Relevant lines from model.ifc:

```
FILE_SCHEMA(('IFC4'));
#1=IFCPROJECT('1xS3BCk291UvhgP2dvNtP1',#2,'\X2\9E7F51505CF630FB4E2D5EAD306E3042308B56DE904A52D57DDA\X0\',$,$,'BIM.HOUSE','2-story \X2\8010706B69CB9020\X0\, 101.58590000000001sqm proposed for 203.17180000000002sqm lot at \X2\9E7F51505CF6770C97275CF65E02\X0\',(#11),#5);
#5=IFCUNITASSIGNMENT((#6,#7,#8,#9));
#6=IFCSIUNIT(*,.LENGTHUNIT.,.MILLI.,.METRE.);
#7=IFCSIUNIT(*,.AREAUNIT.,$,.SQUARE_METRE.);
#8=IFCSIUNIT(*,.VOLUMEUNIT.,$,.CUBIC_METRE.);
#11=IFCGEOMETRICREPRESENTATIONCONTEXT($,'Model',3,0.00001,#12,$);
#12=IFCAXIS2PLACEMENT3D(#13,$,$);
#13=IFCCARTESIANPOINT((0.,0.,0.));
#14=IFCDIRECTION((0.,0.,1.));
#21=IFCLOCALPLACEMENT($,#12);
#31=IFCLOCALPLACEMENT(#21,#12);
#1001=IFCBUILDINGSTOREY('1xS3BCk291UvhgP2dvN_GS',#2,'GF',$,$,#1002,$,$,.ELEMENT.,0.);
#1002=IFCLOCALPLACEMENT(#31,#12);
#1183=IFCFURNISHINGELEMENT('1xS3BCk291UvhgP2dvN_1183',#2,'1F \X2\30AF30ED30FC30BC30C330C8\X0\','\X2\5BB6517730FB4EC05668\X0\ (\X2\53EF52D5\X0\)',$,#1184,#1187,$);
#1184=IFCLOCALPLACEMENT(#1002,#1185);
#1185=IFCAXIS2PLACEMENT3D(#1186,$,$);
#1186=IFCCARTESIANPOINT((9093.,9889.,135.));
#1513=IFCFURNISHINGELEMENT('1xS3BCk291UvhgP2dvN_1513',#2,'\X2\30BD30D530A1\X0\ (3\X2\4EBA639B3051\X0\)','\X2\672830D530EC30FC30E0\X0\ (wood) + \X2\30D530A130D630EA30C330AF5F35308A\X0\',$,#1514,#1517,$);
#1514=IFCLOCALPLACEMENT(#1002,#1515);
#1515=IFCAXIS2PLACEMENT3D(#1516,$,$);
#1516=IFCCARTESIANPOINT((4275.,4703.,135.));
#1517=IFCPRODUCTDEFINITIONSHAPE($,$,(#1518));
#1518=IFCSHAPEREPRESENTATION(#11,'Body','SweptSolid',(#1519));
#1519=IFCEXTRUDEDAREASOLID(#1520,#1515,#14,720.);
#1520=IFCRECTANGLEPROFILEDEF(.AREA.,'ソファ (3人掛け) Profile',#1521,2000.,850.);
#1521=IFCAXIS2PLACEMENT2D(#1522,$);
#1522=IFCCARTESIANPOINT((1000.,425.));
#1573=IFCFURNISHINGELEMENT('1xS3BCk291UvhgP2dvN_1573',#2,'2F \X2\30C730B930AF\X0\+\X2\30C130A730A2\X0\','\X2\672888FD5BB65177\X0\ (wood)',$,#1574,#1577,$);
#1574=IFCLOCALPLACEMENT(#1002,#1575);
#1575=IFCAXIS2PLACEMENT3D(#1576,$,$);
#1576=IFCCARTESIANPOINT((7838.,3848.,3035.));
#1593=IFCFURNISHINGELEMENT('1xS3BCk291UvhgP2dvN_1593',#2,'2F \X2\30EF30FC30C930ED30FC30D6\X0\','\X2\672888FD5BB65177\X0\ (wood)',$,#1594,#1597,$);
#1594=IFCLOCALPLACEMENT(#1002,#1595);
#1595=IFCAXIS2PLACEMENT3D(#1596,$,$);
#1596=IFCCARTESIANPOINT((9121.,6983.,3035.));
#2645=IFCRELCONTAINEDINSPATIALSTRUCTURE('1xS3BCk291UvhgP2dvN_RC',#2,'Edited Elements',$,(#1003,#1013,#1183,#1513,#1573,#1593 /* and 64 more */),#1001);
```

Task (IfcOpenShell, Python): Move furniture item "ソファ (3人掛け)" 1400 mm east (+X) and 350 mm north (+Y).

```python
import ifcopenshell
import ifcopenshell.api.geometry
import ifcopenshell.util.placement
import ifcopenshell.util.unit

model = ifcopenshell.open("model.ifc")
unit_scale = ifcopenshell.util.unit.calculate_unit_scale(model)

item = model.by_id(1513)
matrix = ifcopenshell.util.placement.get_local_placement(item.ObjectPlacement)
matrix[0, 3] += 1.4 / unit_scale
matrix[1, 3] += 0.35 / unit_scale
ifcopenshell.api.geometry.edit_object_placement(model, product=item, matrix=matrix, is_si=False)

print(ifcopenshell.util.placement.get_local_placement(item.ObjectPlacement).round(3) + 0.0)

model.write("model_updated.ifc")
```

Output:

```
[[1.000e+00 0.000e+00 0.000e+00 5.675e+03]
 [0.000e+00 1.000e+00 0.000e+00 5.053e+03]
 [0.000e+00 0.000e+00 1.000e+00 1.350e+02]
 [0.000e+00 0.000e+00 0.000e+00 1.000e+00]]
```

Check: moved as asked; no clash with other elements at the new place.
